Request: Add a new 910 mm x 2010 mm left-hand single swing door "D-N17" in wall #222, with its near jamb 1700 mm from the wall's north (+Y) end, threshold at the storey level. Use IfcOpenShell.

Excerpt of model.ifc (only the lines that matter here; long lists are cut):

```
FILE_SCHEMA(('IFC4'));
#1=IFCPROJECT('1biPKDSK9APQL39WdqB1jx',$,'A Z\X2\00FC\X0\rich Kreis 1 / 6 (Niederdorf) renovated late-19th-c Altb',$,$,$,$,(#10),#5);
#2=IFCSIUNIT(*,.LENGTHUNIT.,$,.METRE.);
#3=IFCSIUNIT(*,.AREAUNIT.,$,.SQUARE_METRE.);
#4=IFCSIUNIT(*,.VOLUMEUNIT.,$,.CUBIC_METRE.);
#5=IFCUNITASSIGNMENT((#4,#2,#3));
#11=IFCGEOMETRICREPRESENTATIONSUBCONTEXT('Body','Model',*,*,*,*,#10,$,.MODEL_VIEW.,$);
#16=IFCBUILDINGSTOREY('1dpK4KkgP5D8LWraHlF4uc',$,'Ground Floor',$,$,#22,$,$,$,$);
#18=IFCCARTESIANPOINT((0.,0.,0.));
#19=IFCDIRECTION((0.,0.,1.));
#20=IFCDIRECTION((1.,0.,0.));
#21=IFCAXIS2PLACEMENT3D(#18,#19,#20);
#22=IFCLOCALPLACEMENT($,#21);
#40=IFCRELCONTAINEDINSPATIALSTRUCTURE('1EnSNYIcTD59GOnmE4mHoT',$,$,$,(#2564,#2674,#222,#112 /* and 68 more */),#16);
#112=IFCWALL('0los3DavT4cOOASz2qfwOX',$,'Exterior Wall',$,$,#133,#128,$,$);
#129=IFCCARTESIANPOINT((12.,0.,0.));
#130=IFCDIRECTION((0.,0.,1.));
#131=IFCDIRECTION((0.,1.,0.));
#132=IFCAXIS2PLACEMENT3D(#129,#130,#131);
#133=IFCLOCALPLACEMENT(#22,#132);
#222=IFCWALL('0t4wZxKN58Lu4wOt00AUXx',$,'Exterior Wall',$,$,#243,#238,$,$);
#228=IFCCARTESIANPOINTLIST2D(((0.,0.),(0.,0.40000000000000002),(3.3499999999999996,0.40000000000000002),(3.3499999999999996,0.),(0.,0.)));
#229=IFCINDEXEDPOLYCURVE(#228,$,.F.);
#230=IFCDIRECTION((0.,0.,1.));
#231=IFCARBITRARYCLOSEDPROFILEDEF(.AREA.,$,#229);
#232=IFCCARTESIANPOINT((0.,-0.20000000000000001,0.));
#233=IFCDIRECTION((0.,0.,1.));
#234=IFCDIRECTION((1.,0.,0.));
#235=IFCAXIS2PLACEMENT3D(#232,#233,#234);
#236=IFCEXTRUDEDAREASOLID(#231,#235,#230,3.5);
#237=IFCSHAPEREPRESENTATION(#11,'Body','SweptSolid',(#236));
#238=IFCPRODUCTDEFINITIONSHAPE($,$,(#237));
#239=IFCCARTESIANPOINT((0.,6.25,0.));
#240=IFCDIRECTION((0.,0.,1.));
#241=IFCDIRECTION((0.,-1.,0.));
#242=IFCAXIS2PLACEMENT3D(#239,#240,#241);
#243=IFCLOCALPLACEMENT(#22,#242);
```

```python
import numpy as np
import ifcopenshell
import ifcopenshell.api.feature
import ifcopenshell.api.geometry
import ifcopenshell.api.root
import ifcopenshell.api.spatial
import ifcopenshell.geom
import ifcopenshell.util.element
import ifcopenshell.util.placement
import ifcopenshell.util.representation
import ifcopenshell.util.shape
import ifcopenshell.util.unit

model = ifcopenshell.open("model.ifc")
unit_scale = ifcopenshell.util.unit.calculate_unit_scale(model)
settings = ifcopenshell.geom.settings()


def volume(element):
    """Net volume in cubic metres, openings subtracted."""
    shape = ifcopenshell.geom.create_shape(settings, element)
    return ifcopenshell.util.shape.get_volume(shape.geometry)


wall = model.by_id(222)
storey = ifcopenshell.util.element.get_container(wall, ifc_class="IfcBuildingStorey")
context = ifcopenshell.util.representation.get_context(model, "Model", "Body", "MODEL_VIEW")
before = volume(wall)

width, height, from_end, sill = 0.91, 2.01, 1.7, 0.0  # metres

# The wall runs along its own X axis, and the end named is its -X end.
wall_shape = ifcopenshell.geom.create_shape(settings, wall)
x, y, z = ifcopenshell.util.shape.get_vertices(wall_shape.geometry).T
start = x.min() + from_end
face, thickness = float(y.min()), float(y.max() - y.min())
wall_matrix = ifcopenshell.util.placement.get_local_placement(wall.ObjectPlacement)
level = ifcopenshell.util.placement.get_local_placement(storey.ObjectPlacement)[2, 3]


def in_wall(x, y):
    """Placement at x, y metres in the wall's axes, at sill height."""
    matrix = wall_matrix.copy()
    matrix[:, 3] = wall_matrix @ np.array([x / unit_scale, y / unit_scale, 0.0, 1.0])
    matrix[2, 3] = level + sill / unit_scale
    return matrix


# Opening: a box that overshoots both wall faces by 50 mm.
opening = ifcopenshell.api.root.create_entity(model, ifc_class="IfcOpeningElement", predefined_type="OPENING")
box = ifcopenshell.api.geometry.add_wall_representation(
    model, context=context, length=width, height=height, thickness=thickness + 0.1
)
ifcopenshell.api.geometry.assign_representation(model, product=opening, representation=box)
ifcopenshell.api.geometry.edit_object_placement(model, product=opening, matrix=in_wall(start, face - 0.05), is_si=False)
ifcopenshell.api.feature.add_feature(model, feature=opening, element=wall)

door = ifcopenshell.api.root.create_entity(model, ifc_class="IfcDoor", name="D-N17", predefined_type="DOOR")
door.OverallWidth, door.OverallHeight = width / unit_scale, height / unit_scale
door.OperationType = "SINGLE_SWING_LEFT"
body = ifcopenshell.api.geometry.add_door_representation(
    model,
    context=context,
    overall_width=door.OverallWidth,
    overall_height=door.OverallHeight,
    operation_type="SINGLE_SWING_LEFT",
    lining_properties={"LiningDepth": thickness / unit_scale, "ThresholdDepth": thickness / unit_scale},
)
ifcopenshell.api.geometry.assign_representation(model, product=door, representation=body)
ifcopenshell.api.spatial.assign_container(model, products=[door], relating_structure=storey)
ifcopenshell.api.feature.add_filling(model, opening=opening, element=door)

# The lining spans the wall, so the door starts at the wall face.
ifcopenshell.api.geometry.edit_object_placement(model, product=door, matrix=in_wall(start, face), is_si=False)

after = volume(wall)

print(f"wall volume {before:.3f} -> {after:.3f} m3")

model.write("model-out.ifc")
```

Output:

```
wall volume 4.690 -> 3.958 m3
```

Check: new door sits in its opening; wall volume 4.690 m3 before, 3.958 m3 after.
